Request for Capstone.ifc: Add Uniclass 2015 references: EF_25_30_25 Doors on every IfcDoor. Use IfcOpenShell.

First a look at what the model holds.

```python
import ifcopenshell

model = ifcopenshell.open("Capstone.ifc")
print(model.schema)
print("classifications:", [c.Name for c in model.by_type("IfcClassification")])
for ifc_class in ("IfcDoor", "IfcRoof", "IfcStair", "IfcWall", "IfcWindow"):
    print(ifc_class, len(model.by_type(ifc_class)))
```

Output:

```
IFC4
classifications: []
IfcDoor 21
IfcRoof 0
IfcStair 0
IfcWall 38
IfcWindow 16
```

```python
import ifcopenshell
import ifcopenshell.api.classification

model = ifcopenshell.open("Capstone.ifc")

system = ifcopenshell.api.classification.add_classification(model, classification="Uniclass 2015")

codes = {
    "IfcDoor": ("EF_25_30_25", "Doors"),
}
for ifc_class, (code, name) in codes.items():
    products = model.by_type(ifc_class)
    ifcopenshell.api.classification.add_reference(
        model, products=products, classification=system, identification=code, name=name
    )
    print(code, len(products))

model.write("Capstone_updated.ifc")
```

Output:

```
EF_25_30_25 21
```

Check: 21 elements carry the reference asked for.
